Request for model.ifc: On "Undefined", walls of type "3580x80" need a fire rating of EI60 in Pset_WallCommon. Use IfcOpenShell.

First a look at what the model holds.

```python
import ifcopenshell
import ifcopenshell.util.element

model = ifcopenshell.open("model.ifc")
print(model.schema)
storey = next(s for s in model.by_type("IfcBuildingStorey") if s.Name == "Undefined")
walls = [e for e in ifcopenshell.util.element.get_decomposition(storey) if e.is_a("IfcWall")]
seen = {}
for e in walls:
    element_type = ifcopenshell.util.element.get_type(e)
    key = (element_type.Name if element_type != e and element_type else None, ifcopenshell.util.element.get_pset(e, "Pset_WallCommon", "FireRating"))
    seen[key] = seen.get(key, 0) + 1
for (name, value), count in sorted(seen.items(), key=str):
    print(count, "x", name, "|", value)
```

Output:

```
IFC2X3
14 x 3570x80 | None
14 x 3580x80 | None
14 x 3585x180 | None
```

```python
import ifcopenshell
import ifcopenshell.api.pset
import ifcopenshell.util.element

model = ifcopenshell.open("model.ifc")

storey = next(s for s in model.by_type("IfcBuildingStorey") if s.Name == "Undefined")
walls = [e for e in ifcopenshell.util.element.get_decomposition(storey) if e.is_a("IfcWall")]

count = 0
for e in walls:
    element_type = ifcopenshell.util.element.get_type(e)
    if element_type in (None, e) or element_type.Name != "3580x80":
        continue
    found = ifcopenshell.util.element.get_pset(e, "Pset_WallCommon", should_inherit=False)
    if found:
        pset = model.by_id(found["id"])
        if len(ifcopenshell.util.element.get_elements_by_pset(pset)) > 1:
            pset = ifcopenshell.api.pset.unshare_pset(model, products=[e], pset=pset)[0]
    else:
        pset = ifcopenshell.api.pset.add_pset(model, product=e, name="Pset_WallCommon")
    ifcopenshell.api.pset.edit_pset(model, pset=pset, properties={"FireRating": "EI60"})
    count += 1

print(count, "walls updated")

model.write("model-out.ifc")
```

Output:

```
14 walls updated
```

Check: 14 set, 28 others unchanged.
